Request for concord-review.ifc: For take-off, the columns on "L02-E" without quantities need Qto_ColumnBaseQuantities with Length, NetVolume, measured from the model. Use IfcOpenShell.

First a look at what the model holds.

```python
import ifcopenshell
import ifcopenshell.util.element
import ifcopenshell.util.unit

model = ifcopenshell.open("concord-review.ifc")
print(model.schema)
for unit_type in ("LENGTHUNIT", "AREAUNIT", "VOLUMEUNIT"):
    print(unit_type, ifcopenshell.util.unit.calculate_unit_scale(model, unit_type))
storey = next(s for s in model.by_type("IfcBuildingStorey") if s.Name == "L02-E")
columns = [e for e in ifcopenshell.util.element.get_decomposition(storey) if e.is_a("IfcColumn")]
for e in sorted(columns, key=lambda e: e.id()):
    print(e.id(), e.is_a(), e.Name, list(ifcopenshell.util.element.get_psets(e, qtos_only=True)), sep=" | ")
```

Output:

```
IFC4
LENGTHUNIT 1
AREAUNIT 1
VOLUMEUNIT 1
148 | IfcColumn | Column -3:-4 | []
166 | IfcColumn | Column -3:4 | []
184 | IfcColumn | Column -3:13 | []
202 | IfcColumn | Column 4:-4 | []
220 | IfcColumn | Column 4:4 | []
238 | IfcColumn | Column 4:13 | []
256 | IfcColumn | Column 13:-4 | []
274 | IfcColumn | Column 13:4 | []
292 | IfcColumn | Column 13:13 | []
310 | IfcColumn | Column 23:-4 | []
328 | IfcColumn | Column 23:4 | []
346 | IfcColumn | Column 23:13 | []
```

```python
import ifcopenshell
import ifcopenshell.api.pset
import ifcopenshell.geom
import ifcopenshell.util.element
import ifcopenshell.util.shape
import ifcopenshell.util.unit

model = ifcopenshell.open("concord-review.ifc")
unit_scale = ifcopenshell.util.unit.calculate_unit_scale(model)
volume_scale = ifcopenshell.util.unit.calculate_unit_scale(model, "VOLUMEUNIT")
settings = ifcopenshell.geom.settings()

storey = next(s for s in model.by_type("IfcBuildingStorey") if s.Name == "L02-E")
columns = [e for e in ifcopenshell.util.element.get_decomposition(storey) if e.is_a("IfcColumn")]

for e in sorted(columns, key=lambda e: e.id()):
    if ifcopenshell.util.element.get_psets(e, qtos_only=True, should_inherit=False):
        continue
    # Geometry comes back in metres, in the element's own axes.
    shape = ifcopenshell.geom.create_shape(settings, e)
    values = {
        "Length": ifcopenshell.util.shape.get_z(shape.geometry) / unit_scale,
        "NetVolume": ifcopenshell.util.shape.get_volume(shape.geometry) / volume_scale,
    }
    qto = ifcopenshell.api.pset.add_qto(model, product=e, name="Qto_ColumnBaseQuantities")
    ifcopenshell.api.pset.edit_qto(model, qto=qto, properties=values)
    print(e.id(), {k: round(v, 3) for k, v in values.items()})

model.write("concord-review-out.ifc")
```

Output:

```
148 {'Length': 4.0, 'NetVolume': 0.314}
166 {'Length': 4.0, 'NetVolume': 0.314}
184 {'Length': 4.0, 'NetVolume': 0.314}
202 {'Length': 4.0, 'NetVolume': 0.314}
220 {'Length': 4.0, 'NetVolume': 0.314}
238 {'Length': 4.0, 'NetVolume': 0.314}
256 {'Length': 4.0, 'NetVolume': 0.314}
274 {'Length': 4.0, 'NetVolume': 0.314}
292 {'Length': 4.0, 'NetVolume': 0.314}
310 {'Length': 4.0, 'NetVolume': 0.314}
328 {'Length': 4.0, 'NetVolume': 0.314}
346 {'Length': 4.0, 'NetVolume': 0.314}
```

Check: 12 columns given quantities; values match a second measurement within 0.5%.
